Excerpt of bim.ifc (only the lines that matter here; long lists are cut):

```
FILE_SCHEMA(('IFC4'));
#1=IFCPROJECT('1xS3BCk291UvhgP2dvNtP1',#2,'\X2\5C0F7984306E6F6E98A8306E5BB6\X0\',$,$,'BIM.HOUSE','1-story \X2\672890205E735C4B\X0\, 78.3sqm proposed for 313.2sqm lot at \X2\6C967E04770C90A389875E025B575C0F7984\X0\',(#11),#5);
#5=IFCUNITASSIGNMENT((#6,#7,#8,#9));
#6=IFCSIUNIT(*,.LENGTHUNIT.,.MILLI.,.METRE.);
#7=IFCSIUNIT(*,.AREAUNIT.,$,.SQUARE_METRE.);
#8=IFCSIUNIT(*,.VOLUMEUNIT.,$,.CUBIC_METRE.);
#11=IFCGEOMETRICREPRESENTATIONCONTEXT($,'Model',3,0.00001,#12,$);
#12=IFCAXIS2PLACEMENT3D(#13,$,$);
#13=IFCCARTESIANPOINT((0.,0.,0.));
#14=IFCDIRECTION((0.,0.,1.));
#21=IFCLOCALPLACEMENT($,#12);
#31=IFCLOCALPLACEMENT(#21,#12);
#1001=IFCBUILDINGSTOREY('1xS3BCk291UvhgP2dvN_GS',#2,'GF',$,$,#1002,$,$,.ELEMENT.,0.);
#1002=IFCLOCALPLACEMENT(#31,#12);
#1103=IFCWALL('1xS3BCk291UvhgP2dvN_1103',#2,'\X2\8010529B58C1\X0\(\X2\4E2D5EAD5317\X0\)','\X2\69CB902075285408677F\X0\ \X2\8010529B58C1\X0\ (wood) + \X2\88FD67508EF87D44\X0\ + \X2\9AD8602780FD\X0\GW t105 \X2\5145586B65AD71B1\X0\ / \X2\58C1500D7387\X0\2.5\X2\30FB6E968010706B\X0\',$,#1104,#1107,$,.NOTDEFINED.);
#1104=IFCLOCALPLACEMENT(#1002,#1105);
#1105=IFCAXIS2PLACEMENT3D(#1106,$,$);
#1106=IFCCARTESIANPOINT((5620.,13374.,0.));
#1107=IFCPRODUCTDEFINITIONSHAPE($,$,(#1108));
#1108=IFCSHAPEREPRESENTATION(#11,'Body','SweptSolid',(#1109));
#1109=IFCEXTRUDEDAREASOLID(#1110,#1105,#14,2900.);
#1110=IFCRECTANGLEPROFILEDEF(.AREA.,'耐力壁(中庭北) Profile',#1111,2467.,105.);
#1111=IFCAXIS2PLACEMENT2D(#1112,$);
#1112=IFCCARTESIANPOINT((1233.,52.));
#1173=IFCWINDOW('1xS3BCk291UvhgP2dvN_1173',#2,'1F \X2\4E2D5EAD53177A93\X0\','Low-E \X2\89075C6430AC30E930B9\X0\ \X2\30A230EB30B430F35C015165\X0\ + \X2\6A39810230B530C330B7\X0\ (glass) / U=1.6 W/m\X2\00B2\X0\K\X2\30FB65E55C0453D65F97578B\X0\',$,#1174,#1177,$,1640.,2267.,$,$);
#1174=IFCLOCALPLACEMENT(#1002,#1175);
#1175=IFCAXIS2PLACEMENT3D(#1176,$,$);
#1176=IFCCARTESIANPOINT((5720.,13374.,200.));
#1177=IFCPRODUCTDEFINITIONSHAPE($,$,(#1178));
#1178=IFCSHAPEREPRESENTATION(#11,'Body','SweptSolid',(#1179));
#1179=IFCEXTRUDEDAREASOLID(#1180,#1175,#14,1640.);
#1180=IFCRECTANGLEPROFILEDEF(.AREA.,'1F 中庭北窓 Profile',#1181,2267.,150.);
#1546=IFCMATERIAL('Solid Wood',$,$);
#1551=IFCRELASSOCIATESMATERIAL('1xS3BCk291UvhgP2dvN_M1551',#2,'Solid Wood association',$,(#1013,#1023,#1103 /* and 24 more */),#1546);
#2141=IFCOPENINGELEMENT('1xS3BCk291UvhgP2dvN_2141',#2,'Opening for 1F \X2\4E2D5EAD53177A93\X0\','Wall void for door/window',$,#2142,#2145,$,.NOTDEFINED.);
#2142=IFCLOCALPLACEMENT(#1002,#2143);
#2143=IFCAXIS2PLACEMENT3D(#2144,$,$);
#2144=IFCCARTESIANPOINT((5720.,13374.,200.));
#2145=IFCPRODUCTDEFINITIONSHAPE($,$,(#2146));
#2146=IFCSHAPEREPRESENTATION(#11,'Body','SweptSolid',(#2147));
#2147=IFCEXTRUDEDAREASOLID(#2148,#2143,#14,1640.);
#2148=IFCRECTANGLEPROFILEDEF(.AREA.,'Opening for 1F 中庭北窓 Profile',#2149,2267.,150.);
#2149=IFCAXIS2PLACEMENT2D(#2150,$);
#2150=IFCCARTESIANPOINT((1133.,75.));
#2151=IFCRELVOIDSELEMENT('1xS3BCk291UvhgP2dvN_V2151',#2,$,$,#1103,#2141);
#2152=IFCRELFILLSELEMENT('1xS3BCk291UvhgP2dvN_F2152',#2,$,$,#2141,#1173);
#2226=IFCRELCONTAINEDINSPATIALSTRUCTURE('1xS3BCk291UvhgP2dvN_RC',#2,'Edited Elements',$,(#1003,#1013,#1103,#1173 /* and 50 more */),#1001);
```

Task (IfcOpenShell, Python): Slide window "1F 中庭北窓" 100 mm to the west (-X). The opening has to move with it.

```python
import ifcopenshell
import ifcopenshell.api.geometry
import ifcopenshell.util.placement
import ifcopenshell.util.unit

model = ifcopenshell.open("bim.ifc")
unit_scale = ifcopenshell.util.unit.calculate_unit_scale(model)

window = model.by_guid("1xS3BCk291UvhgP2dvN_1173")
opening = window.FillsVoids[0].RelatingOpeningElement
wall = opening.VoidsElements[0].RelatingBuildingElement

wall_matrix = ifcopenshell.util.placement.get_local_placement(wall.ObjectPlacement)
shift = wall_matrix[:3, 0] * -0.1 / unit_scale
before = ifcopenshell.util.placement.get_local_placement(window.ObjectPlacement)[:3, 3].copy()

# The window is not placed relative to its opening, so move both.
for product in (opening, window):
    matrix = ifcopenshell.util.placement.get_local_placement(product.ObjectPlacement)
    matrix[:3, 3] += shift
    ifcopenshell.api.geometry.edit_object_placement(model, product=product, matrix=matrix, is_si=False)

after = ifcopenshell.util.placement.get_local_placement(window.ObjectPlacement)[:3, 3]
print("window moved by", (after - before).round(3) + 0.0)

model.write("bim-out.ifc")
```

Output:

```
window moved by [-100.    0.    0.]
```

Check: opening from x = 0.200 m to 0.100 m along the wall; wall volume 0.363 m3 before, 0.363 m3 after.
